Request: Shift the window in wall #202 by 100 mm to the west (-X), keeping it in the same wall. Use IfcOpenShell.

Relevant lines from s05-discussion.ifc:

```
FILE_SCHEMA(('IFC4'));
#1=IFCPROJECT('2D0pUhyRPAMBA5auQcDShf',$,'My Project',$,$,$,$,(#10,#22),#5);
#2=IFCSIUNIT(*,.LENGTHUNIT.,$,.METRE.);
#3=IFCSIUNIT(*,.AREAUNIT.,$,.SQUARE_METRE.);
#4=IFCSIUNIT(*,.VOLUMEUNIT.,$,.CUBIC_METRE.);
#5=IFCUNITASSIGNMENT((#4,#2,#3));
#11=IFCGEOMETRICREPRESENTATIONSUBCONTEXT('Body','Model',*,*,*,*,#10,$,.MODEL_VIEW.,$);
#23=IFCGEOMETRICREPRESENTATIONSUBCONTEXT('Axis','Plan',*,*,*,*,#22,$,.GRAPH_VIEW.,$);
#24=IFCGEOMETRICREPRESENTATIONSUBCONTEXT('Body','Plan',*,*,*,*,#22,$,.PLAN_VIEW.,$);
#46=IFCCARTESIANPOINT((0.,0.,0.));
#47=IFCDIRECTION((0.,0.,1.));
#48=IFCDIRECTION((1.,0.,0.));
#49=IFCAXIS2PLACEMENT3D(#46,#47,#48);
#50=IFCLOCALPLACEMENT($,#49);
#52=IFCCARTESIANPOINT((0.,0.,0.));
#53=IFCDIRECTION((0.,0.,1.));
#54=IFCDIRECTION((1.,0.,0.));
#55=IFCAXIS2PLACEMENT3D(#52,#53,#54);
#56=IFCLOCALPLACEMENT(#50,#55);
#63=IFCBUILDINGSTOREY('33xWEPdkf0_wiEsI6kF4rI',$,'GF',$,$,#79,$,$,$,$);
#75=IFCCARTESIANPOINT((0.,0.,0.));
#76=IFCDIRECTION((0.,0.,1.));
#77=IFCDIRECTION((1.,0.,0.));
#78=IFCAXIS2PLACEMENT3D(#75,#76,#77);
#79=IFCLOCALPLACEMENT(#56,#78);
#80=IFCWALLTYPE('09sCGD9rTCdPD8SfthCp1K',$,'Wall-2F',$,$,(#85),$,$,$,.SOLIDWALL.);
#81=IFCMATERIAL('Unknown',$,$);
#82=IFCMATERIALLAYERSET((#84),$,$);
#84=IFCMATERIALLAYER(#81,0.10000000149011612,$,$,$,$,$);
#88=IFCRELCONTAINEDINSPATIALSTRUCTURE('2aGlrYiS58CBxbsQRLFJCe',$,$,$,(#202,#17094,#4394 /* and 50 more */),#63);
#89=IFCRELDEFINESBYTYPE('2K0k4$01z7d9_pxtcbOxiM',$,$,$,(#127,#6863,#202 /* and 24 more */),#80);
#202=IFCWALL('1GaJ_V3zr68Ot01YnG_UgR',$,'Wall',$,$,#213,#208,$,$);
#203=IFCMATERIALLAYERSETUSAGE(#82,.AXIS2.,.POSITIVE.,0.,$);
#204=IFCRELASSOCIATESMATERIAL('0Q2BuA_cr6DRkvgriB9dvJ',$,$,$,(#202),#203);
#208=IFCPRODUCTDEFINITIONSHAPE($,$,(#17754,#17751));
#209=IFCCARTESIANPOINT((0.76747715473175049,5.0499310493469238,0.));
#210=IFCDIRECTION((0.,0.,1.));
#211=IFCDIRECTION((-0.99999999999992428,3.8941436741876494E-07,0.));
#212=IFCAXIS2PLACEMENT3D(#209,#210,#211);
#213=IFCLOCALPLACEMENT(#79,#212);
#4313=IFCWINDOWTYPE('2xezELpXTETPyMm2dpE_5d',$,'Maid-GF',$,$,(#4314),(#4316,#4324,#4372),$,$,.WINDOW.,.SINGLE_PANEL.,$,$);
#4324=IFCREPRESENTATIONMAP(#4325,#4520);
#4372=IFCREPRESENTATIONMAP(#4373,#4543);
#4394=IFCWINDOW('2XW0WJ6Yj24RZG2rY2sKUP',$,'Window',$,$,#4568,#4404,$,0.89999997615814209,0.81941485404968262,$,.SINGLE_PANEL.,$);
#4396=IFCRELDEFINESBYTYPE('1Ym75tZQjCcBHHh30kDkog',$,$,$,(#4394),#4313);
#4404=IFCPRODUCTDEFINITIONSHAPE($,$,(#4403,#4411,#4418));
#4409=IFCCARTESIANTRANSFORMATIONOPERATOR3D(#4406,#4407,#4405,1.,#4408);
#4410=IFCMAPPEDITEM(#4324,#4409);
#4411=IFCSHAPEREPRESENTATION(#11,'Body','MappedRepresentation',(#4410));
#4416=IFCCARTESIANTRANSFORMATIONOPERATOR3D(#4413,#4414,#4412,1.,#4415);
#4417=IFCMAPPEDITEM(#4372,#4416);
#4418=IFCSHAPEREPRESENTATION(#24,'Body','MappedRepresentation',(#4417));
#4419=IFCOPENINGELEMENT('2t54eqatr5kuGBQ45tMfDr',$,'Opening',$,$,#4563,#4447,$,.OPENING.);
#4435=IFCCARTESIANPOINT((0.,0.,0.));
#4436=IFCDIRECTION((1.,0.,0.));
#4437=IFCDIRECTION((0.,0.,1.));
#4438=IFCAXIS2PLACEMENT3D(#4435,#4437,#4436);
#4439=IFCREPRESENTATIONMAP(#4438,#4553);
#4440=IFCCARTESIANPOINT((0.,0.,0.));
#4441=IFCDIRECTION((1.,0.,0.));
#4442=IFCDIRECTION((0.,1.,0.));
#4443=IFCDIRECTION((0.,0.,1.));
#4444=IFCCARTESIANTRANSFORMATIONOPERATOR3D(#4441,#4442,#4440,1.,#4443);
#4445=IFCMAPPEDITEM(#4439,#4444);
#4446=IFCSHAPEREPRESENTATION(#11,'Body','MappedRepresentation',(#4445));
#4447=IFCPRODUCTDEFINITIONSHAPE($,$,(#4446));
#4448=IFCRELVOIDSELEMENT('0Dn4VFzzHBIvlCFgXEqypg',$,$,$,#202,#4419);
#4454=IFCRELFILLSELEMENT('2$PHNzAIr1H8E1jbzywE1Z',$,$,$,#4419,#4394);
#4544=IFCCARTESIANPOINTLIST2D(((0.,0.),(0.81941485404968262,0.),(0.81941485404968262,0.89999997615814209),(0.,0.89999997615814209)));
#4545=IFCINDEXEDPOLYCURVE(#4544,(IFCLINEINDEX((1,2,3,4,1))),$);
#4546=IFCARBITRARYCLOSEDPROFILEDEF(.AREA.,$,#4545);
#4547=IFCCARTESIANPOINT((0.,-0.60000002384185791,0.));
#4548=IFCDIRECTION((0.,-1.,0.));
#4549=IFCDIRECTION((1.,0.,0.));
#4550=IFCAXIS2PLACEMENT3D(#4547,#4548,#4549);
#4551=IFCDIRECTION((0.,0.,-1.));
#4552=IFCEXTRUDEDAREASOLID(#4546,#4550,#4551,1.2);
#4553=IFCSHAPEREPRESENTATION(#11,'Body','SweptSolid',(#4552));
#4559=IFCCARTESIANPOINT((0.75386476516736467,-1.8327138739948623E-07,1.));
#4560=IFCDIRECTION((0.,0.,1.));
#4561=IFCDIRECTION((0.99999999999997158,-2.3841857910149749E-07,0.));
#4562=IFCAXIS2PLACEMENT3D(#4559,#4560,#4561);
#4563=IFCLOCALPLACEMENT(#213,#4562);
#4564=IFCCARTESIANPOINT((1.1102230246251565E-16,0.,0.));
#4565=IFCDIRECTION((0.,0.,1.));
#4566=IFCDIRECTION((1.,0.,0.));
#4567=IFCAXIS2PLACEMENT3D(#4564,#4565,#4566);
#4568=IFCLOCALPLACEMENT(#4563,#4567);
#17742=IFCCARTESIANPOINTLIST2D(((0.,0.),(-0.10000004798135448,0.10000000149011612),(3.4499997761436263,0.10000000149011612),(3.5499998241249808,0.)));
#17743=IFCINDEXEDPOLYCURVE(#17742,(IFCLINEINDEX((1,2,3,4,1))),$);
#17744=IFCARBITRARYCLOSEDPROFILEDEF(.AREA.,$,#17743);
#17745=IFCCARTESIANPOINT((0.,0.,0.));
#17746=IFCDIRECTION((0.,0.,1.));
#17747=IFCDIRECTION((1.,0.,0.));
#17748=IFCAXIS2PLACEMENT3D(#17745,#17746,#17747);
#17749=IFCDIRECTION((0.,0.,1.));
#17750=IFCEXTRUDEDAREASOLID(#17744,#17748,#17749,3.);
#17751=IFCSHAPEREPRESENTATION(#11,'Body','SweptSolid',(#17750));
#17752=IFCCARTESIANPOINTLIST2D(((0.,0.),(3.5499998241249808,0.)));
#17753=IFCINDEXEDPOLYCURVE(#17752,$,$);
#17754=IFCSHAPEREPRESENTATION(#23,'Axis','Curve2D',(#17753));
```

```python
import ifcopenshell
import ifcopenshell.api.geometry
import ifcopenshell.util.placement
import ifcopenshell.util.unit

model = ifcopenshell.open("s05-discussion.ifc")
unit_scale = ifcopenshell.util.unit.calculate_unit_scale(model)

window = model.by_guid("2XW0WJ6Yj24RZG2rY2sKUP")
opening = window.FillsVoids[0].RelatingOpeningElement
wall = opening.VoidsElements[0].RelatingBuildingElement

wall_matrix = ifcopenshell.util.placement.get_local_placement(wall.ObjectPlacement)
shift = wall_matrix[:3, 0] * 0.1 / unit_scale
before = ifcopenshell.util.placement.get_local_placement(window.ObjectPlacement)[:3, 3].copy()

# The window is placed relative to its opening, so it follows when the opening moves.
matrix = ifcopenshell.util.placement.get_local_placement(opening.ObjectPlacement)
matrix[:3, 3] += shift
ifcopenshell.api.geometry.edit_object_placement(
    model, product=opening, matrix=matrix, is_si=False, should_transform_children=True
)

after = ifcopenshell.util.placement.get_local_placement(window.ObjectPlacement)[:3, 3]
print("window moved by", (after - before).round(3) + 0.0)

model.write("s05-discussion_edited.ifc")
```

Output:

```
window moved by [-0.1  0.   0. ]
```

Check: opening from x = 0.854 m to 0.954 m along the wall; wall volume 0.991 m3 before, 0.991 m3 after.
